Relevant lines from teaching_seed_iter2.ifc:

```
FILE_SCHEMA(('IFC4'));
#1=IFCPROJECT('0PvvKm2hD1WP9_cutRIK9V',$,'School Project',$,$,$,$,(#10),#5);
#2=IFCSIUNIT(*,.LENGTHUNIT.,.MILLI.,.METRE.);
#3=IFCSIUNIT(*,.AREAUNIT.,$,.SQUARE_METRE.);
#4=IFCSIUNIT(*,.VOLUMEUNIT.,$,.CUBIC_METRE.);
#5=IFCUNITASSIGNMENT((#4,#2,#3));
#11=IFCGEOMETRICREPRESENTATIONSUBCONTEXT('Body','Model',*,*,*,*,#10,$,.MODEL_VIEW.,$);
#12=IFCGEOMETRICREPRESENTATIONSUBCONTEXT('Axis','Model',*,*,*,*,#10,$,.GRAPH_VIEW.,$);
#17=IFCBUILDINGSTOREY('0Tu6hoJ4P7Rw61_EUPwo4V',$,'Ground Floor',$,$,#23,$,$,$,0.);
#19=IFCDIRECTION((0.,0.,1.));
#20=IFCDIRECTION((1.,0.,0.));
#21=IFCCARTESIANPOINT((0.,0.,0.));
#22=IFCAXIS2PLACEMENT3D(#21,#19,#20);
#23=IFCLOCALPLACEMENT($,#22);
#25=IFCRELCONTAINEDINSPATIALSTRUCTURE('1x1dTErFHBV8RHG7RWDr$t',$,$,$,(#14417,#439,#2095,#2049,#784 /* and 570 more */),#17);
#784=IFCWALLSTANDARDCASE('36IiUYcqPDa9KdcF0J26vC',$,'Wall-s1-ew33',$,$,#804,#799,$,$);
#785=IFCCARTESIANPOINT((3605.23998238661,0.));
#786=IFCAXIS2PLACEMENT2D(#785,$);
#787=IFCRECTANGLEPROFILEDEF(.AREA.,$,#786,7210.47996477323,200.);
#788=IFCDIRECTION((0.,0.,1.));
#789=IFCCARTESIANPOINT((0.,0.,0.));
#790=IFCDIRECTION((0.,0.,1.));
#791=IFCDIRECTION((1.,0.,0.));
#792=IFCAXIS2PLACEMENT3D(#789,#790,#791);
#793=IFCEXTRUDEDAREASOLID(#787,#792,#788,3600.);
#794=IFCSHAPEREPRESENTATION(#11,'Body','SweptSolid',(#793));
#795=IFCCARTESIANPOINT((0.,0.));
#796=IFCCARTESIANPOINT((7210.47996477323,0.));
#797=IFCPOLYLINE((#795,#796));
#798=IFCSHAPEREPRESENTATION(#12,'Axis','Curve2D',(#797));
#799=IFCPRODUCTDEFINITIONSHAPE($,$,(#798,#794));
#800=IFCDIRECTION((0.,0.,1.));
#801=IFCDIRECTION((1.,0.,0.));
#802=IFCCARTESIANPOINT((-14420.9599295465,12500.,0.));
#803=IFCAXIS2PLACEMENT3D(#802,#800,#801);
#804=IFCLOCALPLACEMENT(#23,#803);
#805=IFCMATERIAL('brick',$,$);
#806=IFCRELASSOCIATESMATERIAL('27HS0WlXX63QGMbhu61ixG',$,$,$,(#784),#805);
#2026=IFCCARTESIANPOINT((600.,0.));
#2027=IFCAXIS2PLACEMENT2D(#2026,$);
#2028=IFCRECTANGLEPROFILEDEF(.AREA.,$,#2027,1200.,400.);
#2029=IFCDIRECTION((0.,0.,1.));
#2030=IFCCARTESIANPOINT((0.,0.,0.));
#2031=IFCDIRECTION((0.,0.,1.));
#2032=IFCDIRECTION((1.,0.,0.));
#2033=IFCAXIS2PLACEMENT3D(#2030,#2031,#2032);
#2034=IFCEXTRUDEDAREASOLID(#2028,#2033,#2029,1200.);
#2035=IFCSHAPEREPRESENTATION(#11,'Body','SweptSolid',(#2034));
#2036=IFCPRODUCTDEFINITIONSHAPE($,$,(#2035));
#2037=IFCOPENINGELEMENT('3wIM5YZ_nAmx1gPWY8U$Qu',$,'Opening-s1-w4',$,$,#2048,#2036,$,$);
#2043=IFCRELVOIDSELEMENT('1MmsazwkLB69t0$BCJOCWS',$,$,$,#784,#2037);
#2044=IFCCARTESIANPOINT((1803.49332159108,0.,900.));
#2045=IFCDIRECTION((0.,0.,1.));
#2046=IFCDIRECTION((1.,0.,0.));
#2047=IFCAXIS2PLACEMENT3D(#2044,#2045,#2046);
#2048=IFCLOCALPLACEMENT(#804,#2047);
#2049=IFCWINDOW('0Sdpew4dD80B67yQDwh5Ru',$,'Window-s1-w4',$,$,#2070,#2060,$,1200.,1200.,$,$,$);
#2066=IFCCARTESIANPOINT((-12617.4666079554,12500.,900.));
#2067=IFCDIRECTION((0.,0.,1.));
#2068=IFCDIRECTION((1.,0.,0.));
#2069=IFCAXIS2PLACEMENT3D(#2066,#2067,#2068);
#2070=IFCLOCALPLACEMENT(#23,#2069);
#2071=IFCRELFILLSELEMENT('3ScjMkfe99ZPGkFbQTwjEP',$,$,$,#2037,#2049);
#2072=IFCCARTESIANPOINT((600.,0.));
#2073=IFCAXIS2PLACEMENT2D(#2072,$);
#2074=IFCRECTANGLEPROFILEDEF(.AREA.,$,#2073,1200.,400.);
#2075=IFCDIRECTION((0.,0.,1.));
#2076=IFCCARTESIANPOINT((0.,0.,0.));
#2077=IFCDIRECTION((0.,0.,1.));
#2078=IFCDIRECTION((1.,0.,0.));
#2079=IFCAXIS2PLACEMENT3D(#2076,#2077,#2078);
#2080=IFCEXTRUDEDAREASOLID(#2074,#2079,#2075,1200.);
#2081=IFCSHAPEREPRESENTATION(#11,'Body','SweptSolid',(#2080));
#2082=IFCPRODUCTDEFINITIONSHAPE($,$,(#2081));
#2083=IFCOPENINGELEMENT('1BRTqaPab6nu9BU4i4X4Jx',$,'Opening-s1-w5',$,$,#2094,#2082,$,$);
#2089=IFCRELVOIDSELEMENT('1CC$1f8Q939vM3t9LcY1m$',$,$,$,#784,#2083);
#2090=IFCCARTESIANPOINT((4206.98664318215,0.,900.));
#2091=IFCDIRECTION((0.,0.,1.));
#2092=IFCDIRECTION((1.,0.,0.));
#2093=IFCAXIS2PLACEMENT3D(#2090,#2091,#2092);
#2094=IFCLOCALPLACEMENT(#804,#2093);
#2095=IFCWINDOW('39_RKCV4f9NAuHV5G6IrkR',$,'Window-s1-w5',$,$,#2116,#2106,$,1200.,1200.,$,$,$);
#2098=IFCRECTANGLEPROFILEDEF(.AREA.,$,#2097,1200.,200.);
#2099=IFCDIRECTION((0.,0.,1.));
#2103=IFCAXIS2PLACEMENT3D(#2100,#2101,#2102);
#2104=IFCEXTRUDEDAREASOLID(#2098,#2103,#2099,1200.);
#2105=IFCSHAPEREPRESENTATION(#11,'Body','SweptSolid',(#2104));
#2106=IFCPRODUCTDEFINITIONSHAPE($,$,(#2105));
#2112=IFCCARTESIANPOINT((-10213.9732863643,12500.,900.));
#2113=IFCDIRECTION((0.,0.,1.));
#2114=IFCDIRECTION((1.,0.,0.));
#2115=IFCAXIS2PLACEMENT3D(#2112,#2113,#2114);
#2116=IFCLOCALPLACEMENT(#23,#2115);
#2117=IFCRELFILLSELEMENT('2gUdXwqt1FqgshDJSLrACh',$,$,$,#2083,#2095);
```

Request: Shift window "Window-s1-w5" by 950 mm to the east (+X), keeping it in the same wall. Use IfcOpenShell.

```python
import ifcopenshell
import ifcopenshell.api.geometry
import ifcopenshell.util.placement

model = ifcopenshell.open("teaching_seed_iter2.ifc")

window = model.by_guid("39_RKCV4f9NAuHV5G6IrkR")
opening = window.FillsVoids[0].RelatingOpeningElement
wall = opening.VoidsElements[0].RelatingBuildingElement

wall_matrix = ifcopenshell.util.placement.get_local_placement(wall.ObjectPlacement)
shift = wall_matrix[:3, 0] * 950.0
before = ifcopenshell.util.placement.get_local_placement(window.ObjectPlacement)[:3, 3].copy()

# The window is not placed relative to its opening, so move both.
for product in (opening, window):
    matrix = ifcopenshell.util.placement.get_local_placement(product.ObjectPlacement)
    matrix[:3, 3] += shift
    ifcopenshell.api.geometry.edit_object_placement(model, product=product, matrix=matrix, is_si=False)

after = ifcopenshell.util.placement.get_local_placement(window.ObjectPlacement)[:3, 3]
print("window moved by", (after - before).round(3) + 0.0)

model.write("teaching_seed_iter2_updated.ifc")
```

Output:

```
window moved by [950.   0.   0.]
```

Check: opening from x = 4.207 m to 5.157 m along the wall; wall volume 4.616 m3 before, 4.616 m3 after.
